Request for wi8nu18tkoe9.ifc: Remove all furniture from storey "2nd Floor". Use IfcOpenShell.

First a look at what the model holds.

```python
import ifcopenshell
import ifcopenshell.util.element

model = ifcopenshell.open("wi8nu18tkoe9.ifc")
print(model.schema)
storey = next(s for s in model.by_type("IfcBuildingStorey") if s.Name == "2nd Floor")
furniture = [e for e in ifcopenshell.util.element.get_decomposition(storey) if e.is_a("IfcFurnishingElement")]
seen = {}
for e in furniture:
    element_type = ifcopenshell.util.element.get_type(e)
    name = element_type.Name if element_type not in (None, e) else None
    seen[name] = seen.get(name, 0) + 1
for name, count in sorted(seen.items(), key=str):
    print(count, "x", name)
```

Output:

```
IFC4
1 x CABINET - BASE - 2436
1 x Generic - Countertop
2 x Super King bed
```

```python
import ifcopenshell
import ifcopenshell.api.root
import ifcopenshell.util.element

model = ifcopenshell.open("wi8nu18tkoe9.ifc")

storey = next(s for s in model.by_type("IfcBuildingStorey") if s.Name == "2nd Floor")
furniture = [e for e in ifcopenshell.util.element.get_decomposition(storey) if e.is_a("IfcFurnishingElement")]

for e in furniture:
    ifcopenshell.api.root.remove_product(model, product=e)
print(len(furniture), "removed")

model.write("wi8nu18tkoe9_rev.ifc")
```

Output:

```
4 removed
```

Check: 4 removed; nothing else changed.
